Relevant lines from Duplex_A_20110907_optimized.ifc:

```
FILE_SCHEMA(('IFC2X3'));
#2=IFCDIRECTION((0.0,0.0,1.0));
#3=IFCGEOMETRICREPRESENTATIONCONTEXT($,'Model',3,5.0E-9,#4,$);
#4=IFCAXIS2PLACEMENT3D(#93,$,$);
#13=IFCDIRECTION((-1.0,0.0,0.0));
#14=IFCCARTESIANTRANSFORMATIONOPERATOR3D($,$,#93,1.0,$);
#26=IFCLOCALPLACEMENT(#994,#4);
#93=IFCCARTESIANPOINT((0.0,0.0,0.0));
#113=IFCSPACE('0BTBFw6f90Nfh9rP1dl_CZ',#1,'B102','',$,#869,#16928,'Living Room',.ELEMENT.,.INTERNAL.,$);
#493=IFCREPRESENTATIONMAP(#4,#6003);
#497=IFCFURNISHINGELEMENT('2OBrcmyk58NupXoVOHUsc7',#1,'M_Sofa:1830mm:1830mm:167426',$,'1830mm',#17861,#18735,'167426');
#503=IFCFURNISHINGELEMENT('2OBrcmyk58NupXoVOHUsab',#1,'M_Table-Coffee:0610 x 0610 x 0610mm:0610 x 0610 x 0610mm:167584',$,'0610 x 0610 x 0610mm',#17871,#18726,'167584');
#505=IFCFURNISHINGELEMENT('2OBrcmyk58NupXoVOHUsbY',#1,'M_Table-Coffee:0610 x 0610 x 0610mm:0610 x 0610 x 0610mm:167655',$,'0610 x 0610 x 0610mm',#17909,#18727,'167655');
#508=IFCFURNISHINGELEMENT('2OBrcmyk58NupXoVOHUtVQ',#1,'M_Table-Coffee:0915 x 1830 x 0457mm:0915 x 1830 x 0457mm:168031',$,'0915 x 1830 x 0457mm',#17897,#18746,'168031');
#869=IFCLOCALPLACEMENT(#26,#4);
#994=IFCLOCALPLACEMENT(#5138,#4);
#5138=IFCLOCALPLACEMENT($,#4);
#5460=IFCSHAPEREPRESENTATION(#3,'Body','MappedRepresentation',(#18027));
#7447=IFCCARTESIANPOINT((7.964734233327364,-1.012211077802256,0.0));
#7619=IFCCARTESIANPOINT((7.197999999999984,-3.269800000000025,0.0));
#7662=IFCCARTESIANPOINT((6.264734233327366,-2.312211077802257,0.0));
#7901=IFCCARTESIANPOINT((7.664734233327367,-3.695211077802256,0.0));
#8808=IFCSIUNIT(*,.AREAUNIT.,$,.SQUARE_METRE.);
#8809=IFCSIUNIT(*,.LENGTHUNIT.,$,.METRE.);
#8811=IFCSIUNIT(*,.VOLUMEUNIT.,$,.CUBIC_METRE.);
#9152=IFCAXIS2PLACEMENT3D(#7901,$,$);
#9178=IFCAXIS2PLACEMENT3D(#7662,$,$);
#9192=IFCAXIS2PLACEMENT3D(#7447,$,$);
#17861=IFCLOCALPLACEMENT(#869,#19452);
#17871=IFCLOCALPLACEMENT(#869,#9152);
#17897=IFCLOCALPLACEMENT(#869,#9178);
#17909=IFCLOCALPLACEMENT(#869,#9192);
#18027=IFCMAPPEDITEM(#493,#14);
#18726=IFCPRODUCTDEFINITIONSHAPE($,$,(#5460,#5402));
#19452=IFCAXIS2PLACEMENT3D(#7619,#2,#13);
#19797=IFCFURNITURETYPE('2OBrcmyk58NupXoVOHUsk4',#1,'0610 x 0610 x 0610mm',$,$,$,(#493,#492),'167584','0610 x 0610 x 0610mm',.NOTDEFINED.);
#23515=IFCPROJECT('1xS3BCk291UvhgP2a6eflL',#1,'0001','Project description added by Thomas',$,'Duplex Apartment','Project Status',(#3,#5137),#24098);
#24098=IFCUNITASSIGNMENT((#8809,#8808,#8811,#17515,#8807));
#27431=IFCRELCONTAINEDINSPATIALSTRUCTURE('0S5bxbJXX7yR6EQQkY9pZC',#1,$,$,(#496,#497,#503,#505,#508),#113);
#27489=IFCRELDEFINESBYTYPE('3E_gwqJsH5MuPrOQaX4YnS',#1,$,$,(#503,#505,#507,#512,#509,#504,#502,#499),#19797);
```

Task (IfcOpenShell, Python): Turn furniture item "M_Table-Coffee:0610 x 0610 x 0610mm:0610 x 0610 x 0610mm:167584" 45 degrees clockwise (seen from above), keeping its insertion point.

```python
import ifcopenshell
import ifcopenshell.api.geometry
import ifcopenshell.util.placement

model = ifcopenshell.open("Duplex_A_20110907_optimized.ifc")

item = model.by_guid("2OBrcmyk58NupXoVOHUsab")
matrix = ifcopenshell.util.placement.get_local_placement(item.ObjectPlacement)
matrix = matrix @ ifcopenshell.util.placement.rotation(-45, "Z")
ifcopenshell.api.geometry.edit_object_placement(model, product=item, matrix=matrix, is_si=False)

print(ifcopenshell.util.placement.get_local_placement(item.ObjectPlacement).round(3) + 0.0)

model.write("Duplex_A_20110907_optimized-out.ifc")
```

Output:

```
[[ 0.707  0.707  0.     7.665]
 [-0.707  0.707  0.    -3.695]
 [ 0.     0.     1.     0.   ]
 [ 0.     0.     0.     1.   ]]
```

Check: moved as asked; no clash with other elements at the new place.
